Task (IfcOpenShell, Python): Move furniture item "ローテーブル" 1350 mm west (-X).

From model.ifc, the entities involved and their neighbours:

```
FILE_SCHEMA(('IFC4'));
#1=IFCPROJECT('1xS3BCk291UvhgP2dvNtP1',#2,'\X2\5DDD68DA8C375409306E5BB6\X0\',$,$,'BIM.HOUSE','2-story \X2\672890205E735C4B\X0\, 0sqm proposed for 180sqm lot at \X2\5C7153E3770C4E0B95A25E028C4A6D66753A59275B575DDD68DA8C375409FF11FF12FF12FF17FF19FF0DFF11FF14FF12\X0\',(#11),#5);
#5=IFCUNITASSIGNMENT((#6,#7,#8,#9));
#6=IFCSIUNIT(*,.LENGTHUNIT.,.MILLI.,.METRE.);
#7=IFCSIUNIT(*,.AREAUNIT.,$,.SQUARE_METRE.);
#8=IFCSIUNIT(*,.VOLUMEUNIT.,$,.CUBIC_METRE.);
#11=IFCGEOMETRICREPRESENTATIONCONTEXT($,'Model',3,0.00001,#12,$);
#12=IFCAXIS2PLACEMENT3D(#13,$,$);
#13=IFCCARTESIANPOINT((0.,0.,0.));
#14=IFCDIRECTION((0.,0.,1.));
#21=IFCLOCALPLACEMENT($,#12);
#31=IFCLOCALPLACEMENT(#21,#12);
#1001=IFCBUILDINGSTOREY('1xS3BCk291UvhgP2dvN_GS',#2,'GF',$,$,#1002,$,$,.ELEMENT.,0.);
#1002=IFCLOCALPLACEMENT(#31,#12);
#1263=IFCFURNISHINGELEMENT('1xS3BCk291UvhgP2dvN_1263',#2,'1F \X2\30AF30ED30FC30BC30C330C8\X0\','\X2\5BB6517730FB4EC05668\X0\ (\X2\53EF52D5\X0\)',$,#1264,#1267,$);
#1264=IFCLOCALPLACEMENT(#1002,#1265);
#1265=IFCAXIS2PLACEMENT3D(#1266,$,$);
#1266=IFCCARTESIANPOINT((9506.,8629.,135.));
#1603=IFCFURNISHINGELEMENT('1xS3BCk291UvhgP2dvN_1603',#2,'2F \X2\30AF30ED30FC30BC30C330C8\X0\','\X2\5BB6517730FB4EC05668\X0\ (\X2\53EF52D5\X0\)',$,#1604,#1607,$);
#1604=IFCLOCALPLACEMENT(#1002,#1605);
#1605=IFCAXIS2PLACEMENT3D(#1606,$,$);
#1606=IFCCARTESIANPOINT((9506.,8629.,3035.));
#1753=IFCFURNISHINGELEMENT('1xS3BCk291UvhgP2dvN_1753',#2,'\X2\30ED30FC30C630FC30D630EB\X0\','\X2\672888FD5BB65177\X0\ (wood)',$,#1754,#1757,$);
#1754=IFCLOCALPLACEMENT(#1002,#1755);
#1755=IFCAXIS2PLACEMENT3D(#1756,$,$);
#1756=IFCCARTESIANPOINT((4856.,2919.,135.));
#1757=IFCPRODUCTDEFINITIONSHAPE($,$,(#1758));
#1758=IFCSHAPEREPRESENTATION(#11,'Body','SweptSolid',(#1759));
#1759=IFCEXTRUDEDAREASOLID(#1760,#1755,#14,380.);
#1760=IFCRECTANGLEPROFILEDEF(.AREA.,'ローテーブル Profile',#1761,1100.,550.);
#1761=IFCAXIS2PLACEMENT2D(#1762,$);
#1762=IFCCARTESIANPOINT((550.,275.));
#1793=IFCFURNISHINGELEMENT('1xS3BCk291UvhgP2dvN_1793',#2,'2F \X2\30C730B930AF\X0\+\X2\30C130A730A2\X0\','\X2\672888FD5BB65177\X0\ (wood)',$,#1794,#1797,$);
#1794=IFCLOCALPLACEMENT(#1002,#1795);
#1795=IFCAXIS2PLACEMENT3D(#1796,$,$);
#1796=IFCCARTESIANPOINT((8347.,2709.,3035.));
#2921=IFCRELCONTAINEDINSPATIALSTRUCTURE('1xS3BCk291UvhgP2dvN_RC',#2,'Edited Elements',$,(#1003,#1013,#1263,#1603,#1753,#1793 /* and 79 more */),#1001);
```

```python
import ifcopenshell
import ifcopenshell.api.geometry
import ifcopenshell.util.placement
import ifcopenshell.util.unit

model = ifcopenshell.open("model.ifc")
unit_scale = ifcopenshell.util.unit.calculate_unit_scale(model)

item = model.by_guid("1xS3BCk291UvhgP2dvN_1753")
matrix = ifcopenshell.util.placement.get_local_placement(item.ObjectPlacement)
matrix[0, 3] -= 1.35 / unit_scale
ifcopenshell.api.geometry.edit_object_placement(model, product=item, matrix=matrix, is_si=False)

print(ifcopenshell.util.placement.get_local_placement(item.ObjectPlacement).round(3) + 0.0)

model.write("model_updated.ifc")
```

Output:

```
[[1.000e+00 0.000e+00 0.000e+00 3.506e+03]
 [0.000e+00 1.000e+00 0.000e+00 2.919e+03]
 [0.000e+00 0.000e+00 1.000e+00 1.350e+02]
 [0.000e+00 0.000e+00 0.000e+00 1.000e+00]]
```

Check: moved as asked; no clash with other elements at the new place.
